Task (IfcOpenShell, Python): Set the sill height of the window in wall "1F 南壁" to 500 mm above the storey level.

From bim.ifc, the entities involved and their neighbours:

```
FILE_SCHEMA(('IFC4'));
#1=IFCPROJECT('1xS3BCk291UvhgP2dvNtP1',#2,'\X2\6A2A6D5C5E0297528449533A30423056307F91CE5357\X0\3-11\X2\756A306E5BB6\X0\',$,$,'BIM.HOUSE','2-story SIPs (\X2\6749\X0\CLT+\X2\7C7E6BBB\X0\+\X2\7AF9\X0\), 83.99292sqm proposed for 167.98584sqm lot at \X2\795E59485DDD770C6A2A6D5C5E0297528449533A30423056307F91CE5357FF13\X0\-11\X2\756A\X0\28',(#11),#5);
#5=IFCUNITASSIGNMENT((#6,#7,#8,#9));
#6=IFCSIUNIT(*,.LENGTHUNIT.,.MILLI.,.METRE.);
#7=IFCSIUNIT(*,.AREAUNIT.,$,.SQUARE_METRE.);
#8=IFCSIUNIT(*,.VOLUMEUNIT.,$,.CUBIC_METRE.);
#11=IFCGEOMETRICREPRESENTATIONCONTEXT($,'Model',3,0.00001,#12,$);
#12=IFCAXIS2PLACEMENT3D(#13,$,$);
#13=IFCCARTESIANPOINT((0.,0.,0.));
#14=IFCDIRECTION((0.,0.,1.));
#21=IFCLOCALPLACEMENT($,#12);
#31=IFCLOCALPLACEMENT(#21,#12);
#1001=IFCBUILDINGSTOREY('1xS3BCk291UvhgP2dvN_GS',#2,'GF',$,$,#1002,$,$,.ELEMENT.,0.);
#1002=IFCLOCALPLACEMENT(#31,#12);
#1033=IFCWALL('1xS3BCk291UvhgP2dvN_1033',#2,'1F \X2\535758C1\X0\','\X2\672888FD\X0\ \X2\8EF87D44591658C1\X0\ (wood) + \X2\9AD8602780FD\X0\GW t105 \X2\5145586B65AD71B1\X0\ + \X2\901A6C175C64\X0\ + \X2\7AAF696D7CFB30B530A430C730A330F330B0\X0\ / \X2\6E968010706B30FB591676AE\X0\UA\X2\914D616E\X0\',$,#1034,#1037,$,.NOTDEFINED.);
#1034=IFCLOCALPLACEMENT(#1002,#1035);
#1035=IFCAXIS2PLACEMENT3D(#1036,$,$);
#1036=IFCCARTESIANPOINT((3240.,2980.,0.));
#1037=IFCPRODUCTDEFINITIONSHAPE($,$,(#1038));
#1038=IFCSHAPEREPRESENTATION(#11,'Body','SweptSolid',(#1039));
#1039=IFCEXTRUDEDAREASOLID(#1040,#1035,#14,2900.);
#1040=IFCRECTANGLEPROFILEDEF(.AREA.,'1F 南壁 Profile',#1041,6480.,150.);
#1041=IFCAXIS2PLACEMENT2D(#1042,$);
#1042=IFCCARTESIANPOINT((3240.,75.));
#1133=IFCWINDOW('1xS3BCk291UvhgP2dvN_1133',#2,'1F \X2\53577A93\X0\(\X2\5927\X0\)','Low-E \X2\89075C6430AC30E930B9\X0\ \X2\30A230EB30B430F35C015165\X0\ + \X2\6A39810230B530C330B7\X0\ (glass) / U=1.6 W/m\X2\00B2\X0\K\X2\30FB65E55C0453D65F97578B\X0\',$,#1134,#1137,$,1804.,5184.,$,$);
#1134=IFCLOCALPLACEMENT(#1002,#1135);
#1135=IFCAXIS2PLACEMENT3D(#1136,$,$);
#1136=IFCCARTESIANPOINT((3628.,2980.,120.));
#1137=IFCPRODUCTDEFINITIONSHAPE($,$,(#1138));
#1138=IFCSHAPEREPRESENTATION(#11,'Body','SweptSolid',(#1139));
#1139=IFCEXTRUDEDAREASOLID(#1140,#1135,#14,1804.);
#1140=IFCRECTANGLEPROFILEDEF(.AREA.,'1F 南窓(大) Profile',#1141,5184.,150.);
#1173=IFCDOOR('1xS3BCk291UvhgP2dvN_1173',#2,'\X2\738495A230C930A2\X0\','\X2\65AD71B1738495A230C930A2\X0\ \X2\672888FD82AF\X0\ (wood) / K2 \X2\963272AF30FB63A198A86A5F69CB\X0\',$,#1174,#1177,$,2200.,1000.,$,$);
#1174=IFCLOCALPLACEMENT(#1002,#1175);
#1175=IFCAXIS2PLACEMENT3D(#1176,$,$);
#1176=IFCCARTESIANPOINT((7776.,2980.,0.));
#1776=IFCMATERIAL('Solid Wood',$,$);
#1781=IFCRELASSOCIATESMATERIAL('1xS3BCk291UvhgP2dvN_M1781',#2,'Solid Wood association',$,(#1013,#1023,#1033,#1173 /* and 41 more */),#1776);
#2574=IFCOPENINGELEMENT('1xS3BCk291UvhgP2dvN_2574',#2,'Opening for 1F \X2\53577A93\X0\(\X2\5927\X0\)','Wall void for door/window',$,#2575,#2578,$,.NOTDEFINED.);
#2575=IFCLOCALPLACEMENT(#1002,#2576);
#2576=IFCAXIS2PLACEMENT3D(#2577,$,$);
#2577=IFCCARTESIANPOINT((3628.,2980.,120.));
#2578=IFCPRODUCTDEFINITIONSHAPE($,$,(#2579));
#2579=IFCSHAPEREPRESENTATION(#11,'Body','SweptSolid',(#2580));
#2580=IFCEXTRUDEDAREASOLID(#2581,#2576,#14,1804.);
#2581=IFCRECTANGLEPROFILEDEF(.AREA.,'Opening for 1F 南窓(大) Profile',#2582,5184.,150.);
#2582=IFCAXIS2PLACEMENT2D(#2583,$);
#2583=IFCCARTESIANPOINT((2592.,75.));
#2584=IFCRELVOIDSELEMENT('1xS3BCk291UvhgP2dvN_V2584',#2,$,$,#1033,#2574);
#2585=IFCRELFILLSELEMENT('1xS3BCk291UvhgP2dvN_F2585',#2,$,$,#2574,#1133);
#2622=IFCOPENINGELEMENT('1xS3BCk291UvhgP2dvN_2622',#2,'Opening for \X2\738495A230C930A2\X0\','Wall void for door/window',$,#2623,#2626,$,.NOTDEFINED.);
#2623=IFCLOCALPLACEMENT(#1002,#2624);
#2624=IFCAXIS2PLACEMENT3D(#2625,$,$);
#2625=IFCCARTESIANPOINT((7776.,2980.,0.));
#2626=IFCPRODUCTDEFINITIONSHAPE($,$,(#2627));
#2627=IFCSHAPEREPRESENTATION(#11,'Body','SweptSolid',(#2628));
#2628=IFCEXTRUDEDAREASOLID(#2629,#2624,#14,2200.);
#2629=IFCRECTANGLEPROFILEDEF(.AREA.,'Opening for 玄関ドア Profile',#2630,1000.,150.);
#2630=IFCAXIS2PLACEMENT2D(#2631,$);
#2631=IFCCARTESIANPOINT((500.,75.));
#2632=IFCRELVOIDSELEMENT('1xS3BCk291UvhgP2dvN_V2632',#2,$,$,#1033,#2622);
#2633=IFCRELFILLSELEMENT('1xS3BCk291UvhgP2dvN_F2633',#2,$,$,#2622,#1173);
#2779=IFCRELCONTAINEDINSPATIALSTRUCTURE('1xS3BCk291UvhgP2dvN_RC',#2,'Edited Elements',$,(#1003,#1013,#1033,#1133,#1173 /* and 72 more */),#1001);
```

```python
import numpy as np
import ifcopenshell
import ifcopenshell.api.geometry
import ifcopenshell.geom
import ifcopenshell.util.element
import ifcopenshell.util.placement
import ifcopenshell.util.shape
import ifcopenshell.util.unit

model = ifcopenshell.open("bim.ifc")
unit_scale = ifcopenshell.util.unit.calculate_unit_scale(model)

window = model.by_guid("1xS3BCk291UvhgP2dvN_1133")
opening = window.FillsVoids[0].RelatingOpeningElement
storey = ifcopenshell.util.element.get_container(window, ifc_class="IfcBuildingStorey")
level = ifcopenshell.util.placement.get_local_placement(storey.ObjectPlacement)[2, 3]

# The opening's origin need not be at the sill, so measure its lowest point.
shape = ifcopenshell.geom.create_shape(ifcopenshell.geom.settings(), opening)
bottom = ifcopenshell.util.shape.get_shape_bottom_elevation(shape, shape.geometry) / unit_scale
dz = level + 0.5 / unit_scale - bottom

shift = np.array([0.0, 0.0, dz])
# The window is not placed relative to its opening, so move both.
for product in (opening, window):
    matrix = ifcopenshell.util.placement.get_local_placement(product.ObjectPlacement)
    matrix[:3, 3] += shift
    ifcopenshell.api.geometry.edit_object_placement(model, product=product, matrix=matrix, is_si=False)

print(f"moved by {dz * unit_scale:+.3f} m")

model.write("bim_edited.ifc")
```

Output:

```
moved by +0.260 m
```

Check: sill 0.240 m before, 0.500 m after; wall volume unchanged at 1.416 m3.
